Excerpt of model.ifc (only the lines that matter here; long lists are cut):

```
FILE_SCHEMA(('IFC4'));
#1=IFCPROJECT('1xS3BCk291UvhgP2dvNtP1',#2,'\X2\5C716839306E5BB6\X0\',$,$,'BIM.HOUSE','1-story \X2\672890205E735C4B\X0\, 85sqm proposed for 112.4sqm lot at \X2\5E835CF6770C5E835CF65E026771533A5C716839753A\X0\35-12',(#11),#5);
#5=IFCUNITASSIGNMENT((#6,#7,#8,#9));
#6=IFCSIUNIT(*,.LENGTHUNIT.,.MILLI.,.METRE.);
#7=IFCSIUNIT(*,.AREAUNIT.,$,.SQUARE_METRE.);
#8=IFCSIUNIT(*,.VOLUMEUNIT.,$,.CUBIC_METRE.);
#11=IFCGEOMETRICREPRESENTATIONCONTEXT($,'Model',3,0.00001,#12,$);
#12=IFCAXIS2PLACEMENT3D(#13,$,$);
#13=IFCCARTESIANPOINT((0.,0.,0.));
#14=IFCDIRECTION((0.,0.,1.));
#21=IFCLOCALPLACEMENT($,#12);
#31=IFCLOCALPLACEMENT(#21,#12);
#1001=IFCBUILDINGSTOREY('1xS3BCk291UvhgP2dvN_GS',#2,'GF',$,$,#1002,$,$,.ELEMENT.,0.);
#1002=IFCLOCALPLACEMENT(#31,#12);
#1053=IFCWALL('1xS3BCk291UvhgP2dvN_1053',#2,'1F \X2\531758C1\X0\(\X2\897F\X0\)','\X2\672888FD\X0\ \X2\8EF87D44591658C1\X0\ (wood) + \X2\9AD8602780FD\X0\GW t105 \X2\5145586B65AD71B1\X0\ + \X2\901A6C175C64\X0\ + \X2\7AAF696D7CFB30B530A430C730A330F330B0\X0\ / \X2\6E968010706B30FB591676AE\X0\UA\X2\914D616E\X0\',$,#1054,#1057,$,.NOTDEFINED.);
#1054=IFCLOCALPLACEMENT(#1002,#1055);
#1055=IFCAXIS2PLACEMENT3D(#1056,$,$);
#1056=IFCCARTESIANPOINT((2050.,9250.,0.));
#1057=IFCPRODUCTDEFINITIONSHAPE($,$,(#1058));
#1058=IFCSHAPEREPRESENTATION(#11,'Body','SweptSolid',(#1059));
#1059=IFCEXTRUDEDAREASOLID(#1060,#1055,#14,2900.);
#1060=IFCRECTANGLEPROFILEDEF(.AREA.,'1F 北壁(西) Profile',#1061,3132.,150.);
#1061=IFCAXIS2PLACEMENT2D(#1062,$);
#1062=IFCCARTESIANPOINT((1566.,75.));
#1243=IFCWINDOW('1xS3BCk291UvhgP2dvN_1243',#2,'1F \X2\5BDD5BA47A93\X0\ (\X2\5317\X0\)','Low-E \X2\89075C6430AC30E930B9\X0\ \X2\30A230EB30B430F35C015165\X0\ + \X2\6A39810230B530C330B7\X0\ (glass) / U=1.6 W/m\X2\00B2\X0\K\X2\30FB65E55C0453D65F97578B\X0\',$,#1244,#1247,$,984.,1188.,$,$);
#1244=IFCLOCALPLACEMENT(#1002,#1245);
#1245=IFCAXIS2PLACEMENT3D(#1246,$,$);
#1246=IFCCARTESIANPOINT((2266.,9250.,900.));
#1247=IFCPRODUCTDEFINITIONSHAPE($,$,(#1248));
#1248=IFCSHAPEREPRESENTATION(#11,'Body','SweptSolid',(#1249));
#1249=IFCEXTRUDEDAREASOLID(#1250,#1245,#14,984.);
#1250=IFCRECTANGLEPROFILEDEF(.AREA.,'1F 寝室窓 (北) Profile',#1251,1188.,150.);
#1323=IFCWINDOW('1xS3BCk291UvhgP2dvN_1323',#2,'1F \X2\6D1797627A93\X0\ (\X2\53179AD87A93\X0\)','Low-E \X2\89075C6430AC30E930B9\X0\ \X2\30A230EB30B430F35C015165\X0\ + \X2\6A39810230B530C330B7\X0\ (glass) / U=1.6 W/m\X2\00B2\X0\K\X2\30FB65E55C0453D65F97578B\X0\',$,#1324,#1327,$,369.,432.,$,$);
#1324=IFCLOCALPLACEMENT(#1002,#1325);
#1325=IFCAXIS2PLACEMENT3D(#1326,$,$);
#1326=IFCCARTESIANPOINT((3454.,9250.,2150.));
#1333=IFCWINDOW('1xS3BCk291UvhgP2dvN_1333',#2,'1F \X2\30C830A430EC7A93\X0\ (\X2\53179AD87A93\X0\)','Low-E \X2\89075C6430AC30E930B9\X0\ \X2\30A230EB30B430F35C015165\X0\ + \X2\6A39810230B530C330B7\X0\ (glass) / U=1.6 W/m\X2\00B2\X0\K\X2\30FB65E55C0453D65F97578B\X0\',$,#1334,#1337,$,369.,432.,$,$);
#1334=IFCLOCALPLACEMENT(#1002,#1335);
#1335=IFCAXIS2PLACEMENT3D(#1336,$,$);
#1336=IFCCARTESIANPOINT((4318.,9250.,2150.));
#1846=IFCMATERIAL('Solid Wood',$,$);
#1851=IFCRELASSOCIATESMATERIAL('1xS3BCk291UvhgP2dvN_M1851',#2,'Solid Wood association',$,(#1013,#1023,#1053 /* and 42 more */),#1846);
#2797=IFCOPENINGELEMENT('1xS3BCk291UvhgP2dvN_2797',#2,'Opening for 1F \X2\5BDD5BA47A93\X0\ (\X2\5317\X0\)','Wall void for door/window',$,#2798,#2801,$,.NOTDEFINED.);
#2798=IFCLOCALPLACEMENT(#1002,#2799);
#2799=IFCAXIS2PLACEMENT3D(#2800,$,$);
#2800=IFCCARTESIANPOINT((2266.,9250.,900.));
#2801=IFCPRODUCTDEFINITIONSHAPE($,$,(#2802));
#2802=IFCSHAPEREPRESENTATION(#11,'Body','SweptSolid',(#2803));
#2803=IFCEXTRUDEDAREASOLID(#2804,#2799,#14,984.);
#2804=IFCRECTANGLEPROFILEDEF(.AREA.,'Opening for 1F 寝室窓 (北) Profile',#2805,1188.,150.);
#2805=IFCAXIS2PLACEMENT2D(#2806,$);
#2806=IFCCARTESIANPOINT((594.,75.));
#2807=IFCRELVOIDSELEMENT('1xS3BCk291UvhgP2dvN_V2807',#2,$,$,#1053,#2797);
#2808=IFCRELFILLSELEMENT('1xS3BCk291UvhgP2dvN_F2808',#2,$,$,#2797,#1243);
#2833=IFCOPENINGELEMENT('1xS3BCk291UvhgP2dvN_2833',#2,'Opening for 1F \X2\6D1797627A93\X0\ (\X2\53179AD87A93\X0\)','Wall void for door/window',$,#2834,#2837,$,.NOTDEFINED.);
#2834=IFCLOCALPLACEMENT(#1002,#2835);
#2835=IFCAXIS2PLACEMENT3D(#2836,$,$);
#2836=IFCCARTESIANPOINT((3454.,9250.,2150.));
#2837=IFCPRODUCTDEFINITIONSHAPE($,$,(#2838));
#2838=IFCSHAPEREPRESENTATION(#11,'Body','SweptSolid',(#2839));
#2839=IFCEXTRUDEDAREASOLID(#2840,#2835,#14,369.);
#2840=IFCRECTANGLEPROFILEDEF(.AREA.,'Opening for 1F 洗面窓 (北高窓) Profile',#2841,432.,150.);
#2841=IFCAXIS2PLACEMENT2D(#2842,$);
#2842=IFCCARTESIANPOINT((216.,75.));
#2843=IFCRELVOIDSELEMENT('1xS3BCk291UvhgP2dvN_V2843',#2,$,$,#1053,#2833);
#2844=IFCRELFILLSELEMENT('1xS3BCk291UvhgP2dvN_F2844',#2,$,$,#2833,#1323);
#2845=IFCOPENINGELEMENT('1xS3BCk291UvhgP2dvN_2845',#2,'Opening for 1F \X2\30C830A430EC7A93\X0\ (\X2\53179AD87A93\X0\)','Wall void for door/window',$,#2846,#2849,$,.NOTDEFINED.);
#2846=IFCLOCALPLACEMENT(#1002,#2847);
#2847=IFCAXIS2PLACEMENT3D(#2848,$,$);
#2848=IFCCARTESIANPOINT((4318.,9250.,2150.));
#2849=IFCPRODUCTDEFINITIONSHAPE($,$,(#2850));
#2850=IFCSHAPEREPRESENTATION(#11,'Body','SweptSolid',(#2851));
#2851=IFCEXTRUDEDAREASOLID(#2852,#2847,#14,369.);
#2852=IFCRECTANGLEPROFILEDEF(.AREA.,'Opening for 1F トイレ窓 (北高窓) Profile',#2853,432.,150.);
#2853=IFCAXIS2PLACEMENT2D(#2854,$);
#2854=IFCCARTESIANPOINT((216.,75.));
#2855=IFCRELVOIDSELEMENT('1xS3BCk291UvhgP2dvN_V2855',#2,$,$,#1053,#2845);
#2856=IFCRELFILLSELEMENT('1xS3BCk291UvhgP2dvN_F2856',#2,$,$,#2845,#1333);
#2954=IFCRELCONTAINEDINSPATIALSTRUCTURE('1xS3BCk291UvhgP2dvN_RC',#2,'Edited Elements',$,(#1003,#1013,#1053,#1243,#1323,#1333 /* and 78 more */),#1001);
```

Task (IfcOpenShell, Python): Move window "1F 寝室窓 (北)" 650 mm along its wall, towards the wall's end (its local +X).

```python
import ifcopenshell
import ifcopenshell.api.geometry
import ifcopenshell.util.placement

model = ifcopenshell.open("model.ifc")

window = model.by_guid("1xS3BCk291UvhgP2dvN_1243")
opening = window.FillsVoids[0].RelatingOpeningElement
wall = opening.VoidsElements[0].RelatingBuildingElement

wall_matrix = ifcopenshell.util.placement.get_local_placement(wall.ObjectPlacement)
shift = wall_matrix[:3, 0] * 650.0
before = ifcopenshell.util.placement.get_local_placement(window.ObjectPlacement)[:3, 3].copy()

# The window is not placed relative to its opening, so move both.
for product in (opening, window):
    matrix = ifcopenshell.util.placement.get_local_placement(product.ObjectPlacement)
    matrix[:3, 3] += shift
    ifcopenshell.api.geometry.edit_object_placement(model, product=product, matrix=matrix, is_si=False)

after = ifcopenshell.util.placement.get_local_placement(window.ObjectPlacement)[:3, 3]
print("window moved by", (after - before).round(3) + 0.0)

model.write("model_updated.ifc")
```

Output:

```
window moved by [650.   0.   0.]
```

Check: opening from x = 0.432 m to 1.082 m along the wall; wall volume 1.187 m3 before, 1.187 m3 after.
